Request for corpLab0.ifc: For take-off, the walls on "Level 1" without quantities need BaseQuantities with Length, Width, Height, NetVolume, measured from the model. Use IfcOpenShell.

First a look at what the model holds.

```python
import ifcopenshell
import ifcopenshell.util.element
import ifcopenshell.util.unit

model = ifcopenshell.open("corpLab0.ifc")
print(model.schema)
for unit_type in ("LENGTHUNIT", "AREAUNIT", "VOLUMEUNIT"):
    print(unit_type, ifcopenshell.util.unit.calculate_unit_scale(model, unit_type))
storey = next(s for s in model.by_type("IfcBuildingStorey") if s.Name == "Level 1")
walls = [e for e in ifcopenshell.util.element.get_decomposition(storey) if e.is_a("IfcWall")]
for e in sorted(walls, key=lambda e: e.id()):
    print(e.id(), e.is_a(), e.Name, list(ifcopenshell.util.element.get_psets(e, qtos_only=True)), sep=" | ")
```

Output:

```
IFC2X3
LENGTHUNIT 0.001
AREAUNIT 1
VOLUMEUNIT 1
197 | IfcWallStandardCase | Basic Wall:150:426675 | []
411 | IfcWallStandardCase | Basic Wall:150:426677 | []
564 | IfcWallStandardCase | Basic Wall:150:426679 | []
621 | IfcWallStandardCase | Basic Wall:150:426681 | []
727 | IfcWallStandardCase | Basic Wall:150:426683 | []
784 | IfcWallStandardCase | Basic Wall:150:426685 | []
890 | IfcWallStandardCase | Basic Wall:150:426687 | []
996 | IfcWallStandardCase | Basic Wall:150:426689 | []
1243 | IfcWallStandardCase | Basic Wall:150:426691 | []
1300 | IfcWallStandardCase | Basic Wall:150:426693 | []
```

```python
import ifcopenshell
import ifcopenshell.api.pset
import ifcopenshell.geom
import ifcopenshell.util.element
import ifcopenshell.util.shape
import ifcopenshell.util.unit

model = ifcopenshell.open("corpLab0.ifc")
unit_scale = ifcopenshell.util.unit.calculate_unit_scale(model)
volume_scale = ifcopenshell.util.unit.calculate_unit_scale(model, "VOLUMEUNIT")
settings = ifcopenshell.geom.settings()

storey = next(s for s in model.by_type("IfcBuildingStorey") if s.Name == "Level 1")
walls = [e for e in ifcopenshell.util.element.get_decomposition(storey) if e.is_a("IfcWall")]

for e in sorted(walls, key=lambda e: e.id()):
    if ifcopenshell.util.element.get_psets(e, qtos_only=True, should_inherit=False):
        continue
    # Geometry comes back in metres, in the element's own axes.
    shape = ifcopenshell.geom.create_shape(settings, e)
    values = {
        "Length": ifcopenshell.util.shape.get_x(shape.geometry) / unit_scale,
        "Width": ifcopenshell.util.shape.get_y(shape.geometry) / unit_scale,
        "Height": ifcopenshell.util.shape.get_z(shape.geometry) / unit_scale,
        "NetVolume": ifcopenshell.util.shape.get_volume(shape.geometry) / volume_scale,
    }
    qto = ifcopenshell.api.pset.add_qto(model, product=e, name="BaseQuantities")
    ifcopenshell.api.pset.edit_qto(model, qto=qto, properties=values)
    print(e.id(), {k: round(v, 3) for k, v in values.items()})

model.write("corpLab0_rev.ifc")
```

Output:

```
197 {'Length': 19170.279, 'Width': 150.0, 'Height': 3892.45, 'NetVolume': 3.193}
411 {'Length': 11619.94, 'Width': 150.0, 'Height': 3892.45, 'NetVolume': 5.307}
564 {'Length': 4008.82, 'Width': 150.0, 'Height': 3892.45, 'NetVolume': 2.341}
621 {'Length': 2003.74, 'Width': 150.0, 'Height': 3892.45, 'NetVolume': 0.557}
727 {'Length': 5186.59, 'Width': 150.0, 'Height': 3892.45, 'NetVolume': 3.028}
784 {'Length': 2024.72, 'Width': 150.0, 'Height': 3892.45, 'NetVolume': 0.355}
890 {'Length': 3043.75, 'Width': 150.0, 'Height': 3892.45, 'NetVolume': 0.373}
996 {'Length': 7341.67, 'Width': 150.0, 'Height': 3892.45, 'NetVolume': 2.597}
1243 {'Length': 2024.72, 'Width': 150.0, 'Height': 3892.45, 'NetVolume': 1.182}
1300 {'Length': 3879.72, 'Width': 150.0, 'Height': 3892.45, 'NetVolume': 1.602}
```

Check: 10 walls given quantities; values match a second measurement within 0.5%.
